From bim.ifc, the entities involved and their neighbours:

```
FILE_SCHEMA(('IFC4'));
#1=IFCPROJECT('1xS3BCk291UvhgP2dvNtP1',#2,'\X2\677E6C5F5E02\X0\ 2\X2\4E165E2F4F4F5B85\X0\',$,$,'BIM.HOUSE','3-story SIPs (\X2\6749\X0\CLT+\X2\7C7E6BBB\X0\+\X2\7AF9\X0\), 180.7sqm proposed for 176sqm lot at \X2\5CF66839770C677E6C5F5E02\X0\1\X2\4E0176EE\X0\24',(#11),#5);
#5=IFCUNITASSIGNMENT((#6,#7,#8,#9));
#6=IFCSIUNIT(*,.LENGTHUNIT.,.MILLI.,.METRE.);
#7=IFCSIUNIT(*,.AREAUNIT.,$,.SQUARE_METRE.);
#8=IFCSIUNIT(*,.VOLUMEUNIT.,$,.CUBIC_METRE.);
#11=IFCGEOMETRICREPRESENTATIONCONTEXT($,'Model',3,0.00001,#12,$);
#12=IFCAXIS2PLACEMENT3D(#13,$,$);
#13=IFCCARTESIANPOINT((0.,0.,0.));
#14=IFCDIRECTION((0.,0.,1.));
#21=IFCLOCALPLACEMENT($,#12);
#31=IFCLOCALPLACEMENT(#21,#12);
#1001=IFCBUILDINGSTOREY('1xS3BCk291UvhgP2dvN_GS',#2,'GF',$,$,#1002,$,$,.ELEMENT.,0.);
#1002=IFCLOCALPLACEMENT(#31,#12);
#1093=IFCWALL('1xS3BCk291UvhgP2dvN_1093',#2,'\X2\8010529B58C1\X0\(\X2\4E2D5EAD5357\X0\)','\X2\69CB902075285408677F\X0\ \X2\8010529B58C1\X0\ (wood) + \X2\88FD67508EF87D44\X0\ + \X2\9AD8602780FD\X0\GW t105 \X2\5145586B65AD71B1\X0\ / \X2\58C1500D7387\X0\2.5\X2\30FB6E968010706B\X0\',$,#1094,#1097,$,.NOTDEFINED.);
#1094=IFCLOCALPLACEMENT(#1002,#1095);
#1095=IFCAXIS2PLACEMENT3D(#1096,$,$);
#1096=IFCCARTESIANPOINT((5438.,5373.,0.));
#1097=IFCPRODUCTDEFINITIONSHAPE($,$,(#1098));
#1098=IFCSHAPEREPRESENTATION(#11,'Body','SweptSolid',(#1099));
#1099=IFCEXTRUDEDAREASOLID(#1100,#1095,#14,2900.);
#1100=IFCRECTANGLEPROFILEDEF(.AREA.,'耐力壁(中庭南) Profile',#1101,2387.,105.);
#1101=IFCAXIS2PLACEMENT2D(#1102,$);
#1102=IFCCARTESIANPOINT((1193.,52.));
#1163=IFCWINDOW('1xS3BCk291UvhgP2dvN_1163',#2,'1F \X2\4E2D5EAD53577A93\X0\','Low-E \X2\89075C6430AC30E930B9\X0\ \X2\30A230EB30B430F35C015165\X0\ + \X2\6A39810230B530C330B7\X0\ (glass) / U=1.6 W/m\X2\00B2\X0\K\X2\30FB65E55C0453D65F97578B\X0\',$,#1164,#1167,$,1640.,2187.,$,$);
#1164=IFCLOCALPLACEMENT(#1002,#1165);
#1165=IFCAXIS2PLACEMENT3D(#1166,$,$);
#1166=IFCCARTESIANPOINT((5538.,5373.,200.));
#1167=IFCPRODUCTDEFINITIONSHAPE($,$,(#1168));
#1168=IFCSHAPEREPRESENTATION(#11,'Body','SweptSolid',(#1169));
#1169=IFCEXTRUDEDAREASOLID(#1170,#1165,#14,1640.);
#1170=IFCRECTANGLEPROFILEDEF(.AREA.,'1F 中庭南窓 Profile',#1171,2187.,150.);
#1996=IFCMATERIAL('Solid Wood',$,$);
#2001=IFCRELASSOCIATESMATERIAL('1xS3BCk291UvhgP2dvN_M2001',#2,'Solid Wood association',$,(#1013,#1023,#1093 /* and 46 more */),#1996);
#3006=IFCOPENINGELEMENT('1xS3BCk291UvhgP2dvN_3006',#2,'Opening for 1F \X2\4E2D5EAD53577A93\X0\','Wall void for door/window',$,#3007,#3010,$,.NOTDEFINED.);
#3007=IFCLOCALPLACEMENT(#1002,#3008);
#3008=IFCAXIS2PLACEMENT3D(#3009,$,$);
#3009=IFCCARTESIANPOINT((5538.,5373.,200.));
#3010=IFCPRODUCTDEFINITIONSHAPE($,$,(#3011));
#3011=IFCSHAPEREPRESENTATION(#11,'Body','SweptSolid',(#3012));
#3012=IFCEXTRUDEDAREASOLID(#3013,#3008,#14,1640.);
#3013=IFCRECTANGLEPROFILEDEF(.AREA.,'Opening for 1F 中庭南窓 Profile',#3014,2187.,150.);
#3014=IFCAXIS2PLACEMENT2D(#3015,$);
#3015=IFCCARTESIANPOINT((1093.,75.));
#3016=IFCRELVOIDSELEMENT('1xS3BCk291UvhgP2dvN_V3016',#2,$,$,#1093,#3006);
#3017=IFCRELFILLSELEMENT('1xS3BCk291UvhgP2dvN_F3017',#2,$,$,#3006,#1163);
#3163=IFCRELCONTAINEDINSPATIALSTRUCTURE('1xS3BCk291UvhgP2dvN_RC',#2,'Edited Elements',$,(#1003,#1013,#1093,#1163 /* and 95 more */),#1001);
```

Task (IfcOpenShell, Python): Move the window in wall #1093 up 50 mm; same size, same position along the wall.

```python
import numpy as np
import ifcopenshell
import ifcopenshell.api.geometry
import ifcopenshell.util.placement
import ifcopenshell.util.unit

model = ifcopenshell.open("bim.ifc")
unit_scale = ifcopenshell.util.unit.calculate_unit_scale(model)

window = model.by_guid("1xS3BCk291UvhgP2dvN_1163")
opening = window.FillsVoids[0].RelatingOpeningElement
dz = 50.0

shift = np.array([0.0, 0.0, dz])
# The window is not placed relative to its opening, so move both.
for product in (opening, window):
    matrix = ifcopenshell.util.placement.get_local_placement(product.ObjectPlacement)
    matrix[:3, 3] += shift
    ifcopenshell.api.geometry.edit_object_placement(model, product=product, matrix=matrix, is_si=False)

print(f"moved by {dz * unit_scale:+.3f} m")

model.write("bim_rev.ifc")
```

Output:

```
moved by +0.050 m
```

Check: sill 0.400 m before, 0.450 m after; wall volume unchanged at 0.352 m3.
